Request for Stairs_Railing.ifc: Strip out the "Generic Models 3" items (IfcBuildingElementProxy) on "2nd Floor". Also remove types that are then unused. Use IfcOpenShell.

First a look at what the model holds.

```python
import ifcopenshell
import ifcopenshell.util.element

model = ifcopenshell.open("Stairs_Railing.ifc")
print(model.schema)
storey = next(s for s in model.by_type("IfcBuildingStorey") if s.Name == "2nd Floor")
proxies = [e for e in ifcopenshell.util.element.get_decomposition(storey) if e.is_a("IfcBuildingElementProxy")]
seen = {}
for e in proxies:
    element_type = ifcopenshell.util.element.get_type(e)
    name = element_type.Name if element_type not in (None, e) else None
    seen[name] = seen.get(name, 0) + 1
for name, count in sorted(seen.items(), key=str):
    print(count, "x", name)
```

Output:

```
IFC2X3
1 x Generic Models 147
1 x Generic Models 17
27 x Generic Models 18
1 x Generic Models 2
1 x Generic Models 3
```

```python
import ifcopenshell
import ifcopenshell.api.root
import ifcopenshell.util.element

model = ifcopenshell.open("Stairs_Railing.ifc")

storey = next(s for s in model.by_type("IfcBuildingStorey") if s.Name == "2nd Floor")
proxies = [e for e in ifcopenshell.util.element.get_decomposition(storey) if e.is_a("IfcBuildingElementProxy")]
targets = [e for e in proxies if (t := ifcopenshell.util.element.get_type(e)) not in (None, e) and t.Name == "Generic Models 3"]
types = {ifcopenshell.util.element.get_type(e) for e in targets} - {None, *targets}

for e in targets:
    ifcopenshell.api.root.remove_product(model, product=e)
print(len(targets), "removed")

unused = [t for t in types if not ifcopenshell.util.element.get_types(t)]
for t in unused:
    ifcopenshell.api.root.remove_product(model, product=t)
print(len(unused), "unused types removed")

model.write("Stairs_Railing_rev.ifc")
```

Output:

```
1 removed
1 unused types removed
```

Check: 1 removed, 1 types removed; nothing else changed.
